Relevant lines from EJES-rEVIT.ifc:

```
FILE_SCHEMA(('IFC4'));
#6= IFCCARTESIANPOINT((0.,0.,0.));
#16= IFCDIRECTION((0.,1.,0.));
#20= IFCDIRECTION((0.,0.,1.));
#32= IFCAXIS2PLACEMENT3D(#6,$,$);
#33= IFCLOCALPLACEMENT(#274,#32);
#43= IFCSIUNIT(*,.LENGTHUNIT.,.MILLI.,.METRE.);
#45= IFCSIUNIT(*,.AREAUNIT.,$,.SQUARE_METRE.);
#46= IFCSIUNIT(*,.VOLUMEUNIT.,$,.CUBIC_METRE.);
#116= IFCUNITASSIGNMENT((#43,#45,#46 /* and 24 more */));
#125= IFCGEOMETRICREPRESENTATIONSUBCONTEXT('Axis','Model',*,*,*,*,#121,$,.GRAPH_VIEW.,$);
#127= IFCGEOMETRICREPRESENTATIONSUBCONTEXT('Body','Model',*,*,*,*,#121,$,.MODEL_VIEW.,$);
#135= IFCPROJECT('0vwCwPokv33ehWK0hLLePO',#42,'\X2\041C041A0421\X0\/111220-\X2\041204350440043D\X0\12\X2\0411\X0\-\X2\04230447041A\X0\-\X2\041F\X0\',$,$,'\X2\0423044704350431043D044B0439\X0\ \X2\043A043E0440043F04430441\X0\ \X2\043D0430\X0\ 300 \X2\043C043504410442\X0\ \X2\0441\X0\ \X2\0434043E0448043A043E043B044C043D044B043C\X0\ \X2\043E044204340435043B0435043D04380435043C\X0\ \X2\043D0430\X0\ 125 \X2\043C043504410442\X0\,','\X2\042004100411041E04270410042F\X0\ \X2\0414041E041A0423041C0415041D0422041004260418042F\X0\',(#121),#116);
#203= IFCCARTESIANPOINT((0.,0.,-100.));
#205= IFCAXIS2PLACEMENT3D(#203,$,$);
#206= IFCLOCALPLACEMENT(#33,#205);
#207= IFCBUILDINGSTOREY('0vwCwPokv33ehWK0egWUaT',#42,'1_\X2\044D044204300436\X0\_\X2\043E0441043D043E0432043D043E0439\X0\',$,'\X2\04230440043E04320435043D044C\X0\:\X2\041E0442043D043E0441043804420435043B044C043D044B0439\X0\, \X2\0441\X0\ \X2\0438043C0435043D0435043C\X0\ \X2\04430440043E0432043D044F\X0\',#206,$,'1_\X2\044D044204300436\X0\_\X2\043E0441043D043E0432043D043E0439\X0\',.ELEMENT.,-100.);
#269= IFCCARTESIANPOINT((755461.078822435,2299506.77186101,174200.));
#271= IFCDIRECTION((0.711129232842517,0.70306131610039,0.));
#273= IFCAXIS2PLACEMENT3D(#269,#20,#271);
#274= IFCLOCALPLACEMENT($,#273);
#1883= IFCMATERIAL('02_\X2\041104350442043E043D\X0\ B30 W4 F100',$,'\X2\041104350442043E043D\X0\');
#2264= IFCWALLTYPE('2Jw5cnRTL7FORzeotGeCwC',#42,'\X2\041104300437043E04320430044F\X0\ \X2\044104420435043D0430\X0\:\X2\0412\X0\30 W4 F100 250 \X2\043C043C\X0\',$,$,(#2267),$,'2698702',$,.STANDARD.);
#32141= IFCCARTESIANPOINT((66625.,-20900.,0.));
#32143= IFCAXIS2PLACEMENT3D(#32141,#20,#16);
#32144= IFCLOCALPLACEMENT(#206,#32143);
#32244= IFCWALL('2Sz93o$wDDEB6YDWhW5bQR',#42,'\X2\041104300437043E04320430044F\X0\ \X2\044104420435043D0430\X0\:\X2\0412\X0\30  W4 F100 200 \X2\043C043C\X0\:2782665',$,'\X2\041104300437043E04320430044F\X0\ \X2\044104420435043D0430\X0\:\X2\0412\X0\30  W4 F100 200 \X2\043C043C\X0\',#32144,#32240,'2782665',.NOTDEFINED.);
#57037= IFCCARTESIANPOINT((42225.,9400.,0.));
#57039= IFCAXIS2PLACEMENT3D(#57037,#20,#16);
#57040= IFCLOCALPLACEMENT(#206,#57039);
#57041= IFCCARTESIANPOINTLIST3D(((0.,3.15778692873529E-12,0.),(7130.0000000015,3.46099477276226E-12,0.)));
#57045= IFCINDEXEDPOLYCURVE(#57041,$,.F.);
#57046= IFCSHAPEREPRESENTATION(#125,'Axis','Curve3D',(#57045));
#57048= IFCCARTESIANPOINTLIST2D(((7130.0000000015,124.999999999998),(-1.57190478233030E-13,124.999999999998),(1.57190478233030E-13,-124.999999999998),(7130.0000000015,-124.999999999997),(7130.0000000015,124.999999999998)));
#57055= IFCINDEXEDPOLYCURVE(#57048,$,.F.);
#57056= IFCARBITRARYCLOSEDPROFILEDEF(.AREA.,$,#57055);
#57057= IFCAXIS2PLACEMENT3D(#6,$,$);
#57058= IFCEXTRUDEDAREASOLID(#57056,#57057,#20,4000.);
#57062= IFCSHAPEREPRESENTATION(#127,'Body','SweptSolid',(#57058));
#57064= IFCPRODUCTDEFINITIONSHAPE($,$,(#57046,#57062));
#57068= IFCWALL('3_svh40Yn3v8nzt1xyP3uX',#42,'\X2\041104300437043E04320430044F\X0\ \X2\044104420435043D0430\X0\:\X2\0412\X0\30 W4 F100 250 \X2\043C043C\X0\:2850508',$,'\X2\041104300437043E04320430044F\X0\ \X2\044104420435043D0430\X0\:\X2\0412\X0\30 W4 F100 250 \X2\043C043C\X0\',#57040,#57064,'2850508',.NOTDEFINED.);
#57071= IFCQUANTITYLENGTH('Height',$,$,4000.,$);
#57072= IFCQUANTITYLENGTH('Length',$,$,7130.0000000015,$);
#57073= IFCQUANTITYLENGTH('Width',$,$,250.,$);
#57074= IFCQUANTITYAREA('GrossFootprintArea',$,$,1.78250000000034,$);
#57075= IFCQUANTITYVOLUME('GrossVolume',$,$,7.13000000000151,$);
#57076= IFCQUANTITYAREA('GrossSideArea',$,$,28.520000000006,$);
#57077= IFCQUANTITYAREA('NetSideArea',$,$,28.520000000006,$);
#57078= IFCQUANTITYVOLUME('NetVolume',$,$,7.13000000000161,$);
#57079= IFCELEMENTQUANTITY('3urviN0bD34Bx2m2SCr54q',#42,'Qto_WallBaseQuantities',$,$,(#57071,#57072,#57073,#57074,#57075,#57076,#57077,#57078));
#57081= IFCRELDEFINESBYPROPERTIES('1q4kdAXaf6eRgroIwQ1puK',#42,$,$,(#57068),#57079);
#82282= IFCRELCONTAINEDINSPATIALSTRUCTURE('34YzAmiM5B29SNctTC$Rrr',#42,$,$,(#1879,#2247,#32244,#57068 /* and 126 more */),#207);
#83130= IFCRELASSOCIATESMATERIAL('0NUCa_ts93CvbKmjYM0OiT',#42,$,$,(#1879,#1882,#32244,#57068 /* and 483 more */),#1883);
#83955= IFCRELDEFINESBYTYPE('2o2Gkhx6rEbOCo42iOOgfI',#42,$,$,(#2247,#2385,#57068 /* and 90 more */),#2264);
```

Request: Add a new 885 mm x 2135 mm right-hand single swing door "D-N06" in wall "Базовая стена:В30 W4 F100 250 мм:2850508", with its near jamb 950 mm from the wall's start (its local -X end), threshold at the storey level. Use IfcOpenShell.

```python
import numpy as np
import ifcopenshell
import ifcopenshell.api.feature
import ifcopenshell.api.geometry
import ifcopenshell.api.pset
import ifcopenshell.api.root
import ifcopenshell.api.spatial
import ifcopenshell.geom
import ifcopenshell.util.element
import ifcopenshell.util.placement
import ifcopenshell.util.representation
import ifcopenshell.util.shape
import ifcopenshell.util.unit

model = ifcopenshell.open("EJES-rEVIT.ifc")
unit_scale = ifcopenshell.util.unit.calculate_unit_scale(model)
area_scale = ifcopenshell.util.unit.calculate_unit_scale(model, "AREAUNIT")
volume_scale = ifcopenshell.util.unit.calculate_unit_scale(model, "VOLUMEUNIT")
settings = ifcopenshell.geom.settings()


def volume(element):
    """Net volume in cubic metres, openings subtracted."""
    shape = ifcopenshell.geom.create_shape(settings, element)
    return ifcopenshell.util.shape.get_volume(shape.geometry)


wall = model.by_guid("3_svh40Yn3v8nzt1xyP3uX")
storey = ifcopenshell.util.element.get_container(wall, ifc_class="IfcBuildingStorey")
context = ifcopenshell.util.representation.get_context(model, "Model", "Body", "MODEL_VIEW")
before = volume(wall)

width, height, from_end, sill = 0.885, 2.135, 0.95, 0.0  # metres

# The wall runs along its own X axis, and the end named is its -X end.
wall_shape = ifcopenshell.geom.create_shape(settings, wall)
x, y, z = ifcopenshell.util.shape.get_vertices(wall_shape.geometry).T
start = x.min() + from_end
face, thickness = float(y.min()), float(y.max() - y.min())
wall_matrix = ifcopenshell.util.placement.get_local_placement(wall.ObjectPlacement)
level = ifcopenshell.util.placement.get_local_placement(storey.ObjectPlacement)[2, 3]


def in_wall(x, y):
    """Placement at x, y metres in the wall's axes, at sill height."""
    matrix = wall_matrix.copy()
    matrix[:, 3] = wall_matrix @ np.array([x / unit_scale, y / unit_scale, 0.0, 1.0])
    matrix[2, 3] = level + sill / unit_scale
    return matrix


# Opening: a box that overshoots both wall faces by 50 mm.
opening = ifcopenshell.api.root.create_entity(model, ifc_class="IfcOpeningElement", predefined_type="OPENING")
box = ifcopenshell.api.geometry.add_wall_representation(
    model, context=context, length=width, height=height, thickness=thickness + 0.1
)
ifcopenshell.api.geometry.assign_representation(model, product=opening, representation=box)
ifcopenshell.api.geometry.edit_object_placement(model, product=opening, matrix=in_wall(start, face - 0.05), is_si=False)
ifcopenshell.api.feature.add_feature(model, feature=opening, element=wall)

door = ifcopenshell.api.root.create_entity(model, ifc_class="IfcDoor", name="D-N06", predefined_type="DOOR")
door.OverallWidth, door.OverallHeight = width / unit_scale, height / unit_scale
door.OperationType = "SINGLE_SWING_RIGHT"
body = ifcopenshell.api.geometry.add_door_representation(
    model,
    context=context,
    overall_width=door.OverallWidth,
    overall_height=door.OverallHeight,
    operation_type="SINGLE_SWING_RIGHT",
    lining_properties={"LiningDepth": thickness / unit_scale, "ThresholdDepth": thickness / unit_scale},
)
ifcopenshell.api.geometry.assign_representation(model, product=door, representation=body)
ifcopenshell.api.spatial.assign_container(model, products=[door], relating_structure=storey)
ifcopenshell.api.feature.add_filling(model, opening=opening, element=door)

# The lining spans the wall, so the door starts at the wall face.
ifcopenshell.api.geometry.edit_object_placement(model, product=door, matrix=in_wall(start, face), is_si=False)

after = volume(wall)

# Update the wall's stored quantities.
qto = model.by_id(ifcopenshell.util.element.get_pset(wall, "Qto_WallBaseQuantities", should_inherit=False)["id"])
ifcopenshell.api.pset.edit_qto(model, qto=qto, properties={
    "NetSideArea": after / thickness / area_scale,
    "NetVolume": after / volume_scale,
})

print(f"wall volume {before:.3f} -> {after:.3f} m3")

model.write("EJES-rEVIT_rev.ifc")
```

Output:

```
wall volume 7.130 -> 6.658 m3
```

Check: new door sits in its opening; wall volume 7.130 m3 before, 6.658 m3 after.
